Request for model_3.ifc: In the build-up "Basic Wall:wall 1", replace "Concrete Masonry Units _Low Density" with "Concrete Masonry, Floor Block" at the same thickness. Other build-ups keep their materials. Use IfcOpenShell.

First a look at what the model holds.

```python
import ifcopenshell
import ifcopenshell.util.element

model = ifcopenshell.open("model_3.ifc")
print(model.schema)
for layer_set in model.by_type("IfcMaterialLayerSet"):
    if layer_set.LayerSetName == "Basic Wall:wall 1":
        for layer in layer_set.MaterialLayers:
            print(layer.id(), layer.Material and layer.Material.Name, layer.LayerThickness, sep=" | ")
        print(len(ifcopenshell.util.element.get_elements_by_material(model, layer_set)), "elements and types use it")
print(sorted(m.Name for m in model.by_type("IfcMaterial") if m.Name)[:60])
```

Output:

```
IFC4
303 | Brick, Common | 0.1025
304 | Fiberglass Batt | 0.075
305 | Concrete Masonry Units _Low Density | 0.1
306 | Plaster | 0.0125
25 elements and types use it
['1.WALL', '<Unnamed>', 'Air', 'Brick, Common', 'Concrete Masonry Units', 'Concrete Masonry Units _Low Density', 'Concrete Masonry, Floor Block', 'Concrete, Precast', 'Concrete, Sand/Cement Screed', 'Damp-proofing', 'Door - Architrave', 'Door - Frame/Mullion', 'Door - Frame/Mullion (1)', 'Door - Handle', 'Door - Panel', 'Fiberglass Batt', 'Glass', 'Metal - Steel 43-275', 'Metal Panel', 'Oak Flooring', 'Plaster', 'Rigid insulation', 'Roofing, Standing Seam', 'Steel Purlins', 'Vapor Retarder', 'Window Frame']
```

```python
import ifcopenshell
import ifcopenshell.api.material

model = ifcopenshell.open("model_3.ifc")

layer_set = next(s for s in model.by_type("IfcMaterialLayerSet") if s.LayerSetName == "Basic Wall:wall 1")
layer = next(l for l in layer_set.MaterialLayers if l.Material and l.Material.Name == "Concrete Masonry Units _Low Density")
material = next(m for m in model.by_type("IfcMaterial") if m.Name == "Concrete Masonry, Floor Block")

# Point this one layer at the other material; renaming the old one would change it everywhere.
ifcopenshell.api.material.edit_layer(model, layer=layer, attributes={"Name": material.Name}, material=material)

print([l.Material.Name if l.Material else None for l in layer_set.MaterialLayers])

model.write("model_3_v2.ifc")
```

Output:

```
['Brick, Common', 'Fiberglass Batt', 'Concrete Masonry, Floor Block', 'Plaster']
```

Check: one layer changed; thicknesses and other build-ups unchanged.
